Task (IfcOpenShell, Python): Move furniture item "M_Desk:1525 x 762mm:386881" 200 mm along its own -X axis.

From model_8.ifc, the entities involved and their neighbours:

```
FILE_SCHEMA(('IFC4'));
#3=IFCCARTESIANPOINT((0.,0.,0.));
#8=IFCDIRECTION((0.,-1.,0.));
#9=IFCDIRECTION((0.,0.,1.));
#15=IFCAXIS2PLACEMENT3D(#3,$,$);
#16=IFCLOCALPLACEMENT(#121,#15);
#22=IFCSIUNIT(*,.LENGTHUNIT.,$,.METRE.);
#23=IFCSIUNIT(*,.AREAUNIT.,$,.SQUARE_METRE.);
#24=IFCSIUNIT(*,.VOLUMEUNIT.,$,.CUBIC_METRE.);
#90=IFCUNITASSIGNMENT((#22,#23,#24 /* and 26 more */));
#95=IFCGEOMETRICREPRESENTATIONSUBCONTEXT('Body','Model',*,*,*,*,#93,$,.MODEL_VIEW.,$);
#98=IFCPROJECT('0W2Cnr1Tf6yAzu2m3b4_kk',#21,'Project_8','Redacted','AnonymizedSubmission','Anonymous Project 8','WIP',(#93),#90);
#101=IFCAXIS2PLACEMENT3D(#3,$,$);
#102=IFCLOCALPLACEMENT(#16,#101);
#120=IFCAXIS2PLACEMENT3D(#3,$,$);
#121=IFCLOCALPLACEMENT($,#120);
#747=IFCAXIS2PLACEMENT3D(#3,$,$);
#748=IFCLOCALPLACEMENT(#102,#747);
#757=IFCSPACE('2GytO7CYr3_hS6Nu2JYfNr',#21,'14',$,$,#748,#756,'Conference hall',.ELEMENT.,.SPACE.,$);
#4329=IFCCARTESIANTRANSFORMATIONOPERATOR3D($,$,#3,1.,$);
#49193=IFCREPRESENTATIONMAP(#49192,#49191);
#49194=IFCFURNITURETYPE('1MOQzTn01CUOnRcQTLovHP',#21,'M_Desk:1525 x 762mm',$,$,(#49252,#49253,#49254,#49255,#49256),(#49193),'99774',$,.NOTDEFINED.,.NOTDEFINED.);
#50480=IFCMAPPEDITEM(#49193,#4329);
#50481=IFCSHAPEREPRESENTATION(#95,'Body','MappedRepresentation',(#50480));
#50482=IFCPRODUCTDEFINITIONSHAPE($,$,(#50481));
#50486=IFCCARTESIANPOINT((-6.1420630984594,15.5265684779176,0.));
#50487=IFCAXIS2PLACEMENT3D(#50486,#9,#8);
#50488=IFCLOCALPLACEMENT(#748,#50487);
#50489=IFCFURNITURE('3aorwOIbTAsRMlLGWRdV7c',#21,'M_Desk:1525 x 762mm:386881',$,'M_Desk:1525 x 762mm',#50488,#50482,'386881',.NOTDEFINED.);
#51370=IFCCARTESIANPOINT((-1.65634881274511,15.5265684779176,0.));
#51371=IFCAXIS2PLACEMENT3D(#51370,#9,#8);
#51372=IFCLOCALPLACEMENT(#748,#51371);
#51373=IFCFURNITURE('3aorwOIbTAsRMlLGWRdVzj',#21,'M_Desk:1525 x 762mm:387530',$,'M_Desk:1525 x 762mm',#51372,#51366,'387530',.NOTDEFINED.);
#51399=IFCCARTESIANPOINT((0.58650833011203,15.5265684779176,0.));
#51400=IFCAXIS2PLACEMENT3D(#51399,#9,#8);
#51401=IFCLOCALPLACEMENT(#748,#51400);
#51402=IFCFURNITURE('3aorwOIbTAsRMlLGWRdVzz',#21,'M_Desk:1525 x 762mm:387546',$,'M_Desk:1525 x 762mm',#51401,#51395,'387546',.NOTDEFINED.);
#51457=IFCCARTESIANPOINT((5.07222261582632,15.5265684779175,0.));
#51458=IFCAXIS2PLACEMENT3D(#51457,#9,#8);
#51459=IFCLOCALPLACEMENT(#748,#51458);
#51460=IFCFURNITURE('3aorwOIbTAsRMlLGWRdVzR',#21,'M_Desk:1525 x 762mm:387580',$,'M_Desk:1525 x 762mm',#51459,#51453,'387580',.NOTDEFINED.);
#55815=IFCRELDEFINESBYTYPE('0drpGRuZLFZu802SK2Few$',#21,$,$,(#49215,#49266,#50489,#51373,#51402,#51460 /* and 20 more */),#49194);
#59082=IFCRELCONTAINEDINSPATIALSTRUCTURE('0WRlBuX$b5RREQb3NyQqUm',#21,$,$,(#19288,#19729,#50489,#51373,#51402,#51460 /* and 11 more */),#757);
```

```python
import ifcopenshell
import ifcopenshell.api.geometry
import ifcopenshell.util.placement
import ifcopenshell.util.unit

model = ifcopenshell.open("model_8.ifc")
unit_scale = ifcopenshell.util.unit.calculate_unit_scale(model)

item = model.by_guid("3aorwOIbTAsRMlLGWRdV7c")
matrix = ifcopenshell.util.placement.get_local_placement(item.ObjectPlacement)
matrix[:3, 3] -= matrix[:3, 0] * 0.2 / unit_scale
ifcopenshell.api.geometry.edit_object_placement(model, product=item, matrix=matrix, is_si=False)

print(ifcopenshell.util.placement.get_local_placement(item.ObjectPlacement).round(3) + 0.0)

model.write("model_8_rev.ifc")
```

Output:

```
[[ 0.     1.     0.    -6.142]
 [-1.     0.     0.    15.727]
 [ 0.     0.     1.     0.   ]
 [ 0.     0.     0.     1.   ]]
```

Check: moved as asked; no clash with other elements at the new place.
